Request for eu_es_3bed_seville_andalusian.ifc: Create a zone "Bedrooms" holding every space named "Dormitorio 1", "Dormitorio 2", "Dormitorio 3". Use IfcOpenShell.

First a look at what the model holds.

```python
import ifcopenshell

model = ifcopenshell.open("eu_es_3bed_seville_andalusian.ifc")
print(model.schema)
seen = {}
for space in model.by_type("IfcSpace"):
    seen[space.LongName] = seen.get(space.LongName, 0) + 1
for name, count in sorted(seen.items(), key=str):
    print(count, "x", name)
print("zones:", [z.Name for z in model.by_type("IfcZone")][:20])
```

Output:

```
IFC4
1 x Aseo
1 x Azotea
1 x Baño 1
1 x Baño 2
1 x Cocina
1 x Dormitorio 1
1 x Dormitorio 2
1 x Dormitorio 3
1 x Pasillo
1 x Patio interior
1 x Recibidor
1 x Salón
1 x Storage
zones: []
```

```python
import ifcopenshell
import ifcopenshell.api.group
import ifcopenshell.api.root

model = ifcopenshell.open("eu_es_3bed_seville_andalusian.ifc")

names = {"Dormitorio 1", "Dormitorio 2", "Dormitorio 3"}
spaces = [s for s in model.by_type("IfcSpace") if s.LongName in names]

zone = ifcopenshell.api.root.create_entity(model, ifc_class="IfcZone", name="Bedrooms")
ifcopenshell.api.group.assign_group(model, products=spaces, group=zone)
print(len(spaces), "spaces in", zone.Name)

model.write("eu_es_3bed_seville_andalusian_edited.ifc")
```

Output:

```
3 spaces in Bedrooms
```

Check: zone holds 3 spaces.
